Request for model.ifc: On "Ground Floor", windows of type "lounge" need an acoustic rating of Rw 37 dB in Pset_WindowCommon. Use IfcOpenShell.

First a look at what the model holds.

```python
import ifcopenshell
import ifcopenshell.util.element

model = ifcopenshell.open("model.ifc")
print(model.schema)
storey = next(s for s in model.by_type("IfcBuildingStorey") if s.Name == "Ground Floor")
windows = [e for e in ifcopenshell.util.element.get_decomposition(storey) if e.is_a("IfcWindow")]
seen = {}
for e in windows:
    element_type = ifcopenshell.util.element.get_type(e)
    key = (element_type.Name if element_type != e and element_type else None, ifcopenshell.util.element.get_pset(e, "Pset_WindowCommon", "AcousticRating"))
    seen[key] = seen.get(key, 0) + 1
for (name, value), count in sorted(seen.items(), key=str):
    print(count, "x", name, "|", value)
```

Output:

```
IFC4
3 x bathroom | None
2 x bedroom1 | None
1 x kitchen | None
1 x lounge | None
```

```python
import ifcopenshell
import ifcopenshell.api.pset
import ifcopenshell.util.element

model = ifcopenshell.open("model.ifc")

storey = next(s for s in model.by_type("IfcBuildingStorey") if s.Name == "Ground Floor")
windows = [e for e in ifcopenshell.util.element.get_decomposition(storey) if e.is_a("IfcWindow")]

count = 0
for e in windows:
    element_type = ifcopenshell.util.element.get_type(e)
    if element_type in (None, e) or element_type.Name != "lounge":
        continue
    # add_pset returns the element's existing set when there is one.
    pset = ifcopenshell.api.pset.add_pset(model, product=e, name="Pset_WindowCommon")
    ifcopenshell.api.pset.edit_pset(model, pset=pset, properties={"AcousticRating": "Rw 37 dB"})
    count += 1

print(count, "windows updated")

model.write("model_rev.ifc")
```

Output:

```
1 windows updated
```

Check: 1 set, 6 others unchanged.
